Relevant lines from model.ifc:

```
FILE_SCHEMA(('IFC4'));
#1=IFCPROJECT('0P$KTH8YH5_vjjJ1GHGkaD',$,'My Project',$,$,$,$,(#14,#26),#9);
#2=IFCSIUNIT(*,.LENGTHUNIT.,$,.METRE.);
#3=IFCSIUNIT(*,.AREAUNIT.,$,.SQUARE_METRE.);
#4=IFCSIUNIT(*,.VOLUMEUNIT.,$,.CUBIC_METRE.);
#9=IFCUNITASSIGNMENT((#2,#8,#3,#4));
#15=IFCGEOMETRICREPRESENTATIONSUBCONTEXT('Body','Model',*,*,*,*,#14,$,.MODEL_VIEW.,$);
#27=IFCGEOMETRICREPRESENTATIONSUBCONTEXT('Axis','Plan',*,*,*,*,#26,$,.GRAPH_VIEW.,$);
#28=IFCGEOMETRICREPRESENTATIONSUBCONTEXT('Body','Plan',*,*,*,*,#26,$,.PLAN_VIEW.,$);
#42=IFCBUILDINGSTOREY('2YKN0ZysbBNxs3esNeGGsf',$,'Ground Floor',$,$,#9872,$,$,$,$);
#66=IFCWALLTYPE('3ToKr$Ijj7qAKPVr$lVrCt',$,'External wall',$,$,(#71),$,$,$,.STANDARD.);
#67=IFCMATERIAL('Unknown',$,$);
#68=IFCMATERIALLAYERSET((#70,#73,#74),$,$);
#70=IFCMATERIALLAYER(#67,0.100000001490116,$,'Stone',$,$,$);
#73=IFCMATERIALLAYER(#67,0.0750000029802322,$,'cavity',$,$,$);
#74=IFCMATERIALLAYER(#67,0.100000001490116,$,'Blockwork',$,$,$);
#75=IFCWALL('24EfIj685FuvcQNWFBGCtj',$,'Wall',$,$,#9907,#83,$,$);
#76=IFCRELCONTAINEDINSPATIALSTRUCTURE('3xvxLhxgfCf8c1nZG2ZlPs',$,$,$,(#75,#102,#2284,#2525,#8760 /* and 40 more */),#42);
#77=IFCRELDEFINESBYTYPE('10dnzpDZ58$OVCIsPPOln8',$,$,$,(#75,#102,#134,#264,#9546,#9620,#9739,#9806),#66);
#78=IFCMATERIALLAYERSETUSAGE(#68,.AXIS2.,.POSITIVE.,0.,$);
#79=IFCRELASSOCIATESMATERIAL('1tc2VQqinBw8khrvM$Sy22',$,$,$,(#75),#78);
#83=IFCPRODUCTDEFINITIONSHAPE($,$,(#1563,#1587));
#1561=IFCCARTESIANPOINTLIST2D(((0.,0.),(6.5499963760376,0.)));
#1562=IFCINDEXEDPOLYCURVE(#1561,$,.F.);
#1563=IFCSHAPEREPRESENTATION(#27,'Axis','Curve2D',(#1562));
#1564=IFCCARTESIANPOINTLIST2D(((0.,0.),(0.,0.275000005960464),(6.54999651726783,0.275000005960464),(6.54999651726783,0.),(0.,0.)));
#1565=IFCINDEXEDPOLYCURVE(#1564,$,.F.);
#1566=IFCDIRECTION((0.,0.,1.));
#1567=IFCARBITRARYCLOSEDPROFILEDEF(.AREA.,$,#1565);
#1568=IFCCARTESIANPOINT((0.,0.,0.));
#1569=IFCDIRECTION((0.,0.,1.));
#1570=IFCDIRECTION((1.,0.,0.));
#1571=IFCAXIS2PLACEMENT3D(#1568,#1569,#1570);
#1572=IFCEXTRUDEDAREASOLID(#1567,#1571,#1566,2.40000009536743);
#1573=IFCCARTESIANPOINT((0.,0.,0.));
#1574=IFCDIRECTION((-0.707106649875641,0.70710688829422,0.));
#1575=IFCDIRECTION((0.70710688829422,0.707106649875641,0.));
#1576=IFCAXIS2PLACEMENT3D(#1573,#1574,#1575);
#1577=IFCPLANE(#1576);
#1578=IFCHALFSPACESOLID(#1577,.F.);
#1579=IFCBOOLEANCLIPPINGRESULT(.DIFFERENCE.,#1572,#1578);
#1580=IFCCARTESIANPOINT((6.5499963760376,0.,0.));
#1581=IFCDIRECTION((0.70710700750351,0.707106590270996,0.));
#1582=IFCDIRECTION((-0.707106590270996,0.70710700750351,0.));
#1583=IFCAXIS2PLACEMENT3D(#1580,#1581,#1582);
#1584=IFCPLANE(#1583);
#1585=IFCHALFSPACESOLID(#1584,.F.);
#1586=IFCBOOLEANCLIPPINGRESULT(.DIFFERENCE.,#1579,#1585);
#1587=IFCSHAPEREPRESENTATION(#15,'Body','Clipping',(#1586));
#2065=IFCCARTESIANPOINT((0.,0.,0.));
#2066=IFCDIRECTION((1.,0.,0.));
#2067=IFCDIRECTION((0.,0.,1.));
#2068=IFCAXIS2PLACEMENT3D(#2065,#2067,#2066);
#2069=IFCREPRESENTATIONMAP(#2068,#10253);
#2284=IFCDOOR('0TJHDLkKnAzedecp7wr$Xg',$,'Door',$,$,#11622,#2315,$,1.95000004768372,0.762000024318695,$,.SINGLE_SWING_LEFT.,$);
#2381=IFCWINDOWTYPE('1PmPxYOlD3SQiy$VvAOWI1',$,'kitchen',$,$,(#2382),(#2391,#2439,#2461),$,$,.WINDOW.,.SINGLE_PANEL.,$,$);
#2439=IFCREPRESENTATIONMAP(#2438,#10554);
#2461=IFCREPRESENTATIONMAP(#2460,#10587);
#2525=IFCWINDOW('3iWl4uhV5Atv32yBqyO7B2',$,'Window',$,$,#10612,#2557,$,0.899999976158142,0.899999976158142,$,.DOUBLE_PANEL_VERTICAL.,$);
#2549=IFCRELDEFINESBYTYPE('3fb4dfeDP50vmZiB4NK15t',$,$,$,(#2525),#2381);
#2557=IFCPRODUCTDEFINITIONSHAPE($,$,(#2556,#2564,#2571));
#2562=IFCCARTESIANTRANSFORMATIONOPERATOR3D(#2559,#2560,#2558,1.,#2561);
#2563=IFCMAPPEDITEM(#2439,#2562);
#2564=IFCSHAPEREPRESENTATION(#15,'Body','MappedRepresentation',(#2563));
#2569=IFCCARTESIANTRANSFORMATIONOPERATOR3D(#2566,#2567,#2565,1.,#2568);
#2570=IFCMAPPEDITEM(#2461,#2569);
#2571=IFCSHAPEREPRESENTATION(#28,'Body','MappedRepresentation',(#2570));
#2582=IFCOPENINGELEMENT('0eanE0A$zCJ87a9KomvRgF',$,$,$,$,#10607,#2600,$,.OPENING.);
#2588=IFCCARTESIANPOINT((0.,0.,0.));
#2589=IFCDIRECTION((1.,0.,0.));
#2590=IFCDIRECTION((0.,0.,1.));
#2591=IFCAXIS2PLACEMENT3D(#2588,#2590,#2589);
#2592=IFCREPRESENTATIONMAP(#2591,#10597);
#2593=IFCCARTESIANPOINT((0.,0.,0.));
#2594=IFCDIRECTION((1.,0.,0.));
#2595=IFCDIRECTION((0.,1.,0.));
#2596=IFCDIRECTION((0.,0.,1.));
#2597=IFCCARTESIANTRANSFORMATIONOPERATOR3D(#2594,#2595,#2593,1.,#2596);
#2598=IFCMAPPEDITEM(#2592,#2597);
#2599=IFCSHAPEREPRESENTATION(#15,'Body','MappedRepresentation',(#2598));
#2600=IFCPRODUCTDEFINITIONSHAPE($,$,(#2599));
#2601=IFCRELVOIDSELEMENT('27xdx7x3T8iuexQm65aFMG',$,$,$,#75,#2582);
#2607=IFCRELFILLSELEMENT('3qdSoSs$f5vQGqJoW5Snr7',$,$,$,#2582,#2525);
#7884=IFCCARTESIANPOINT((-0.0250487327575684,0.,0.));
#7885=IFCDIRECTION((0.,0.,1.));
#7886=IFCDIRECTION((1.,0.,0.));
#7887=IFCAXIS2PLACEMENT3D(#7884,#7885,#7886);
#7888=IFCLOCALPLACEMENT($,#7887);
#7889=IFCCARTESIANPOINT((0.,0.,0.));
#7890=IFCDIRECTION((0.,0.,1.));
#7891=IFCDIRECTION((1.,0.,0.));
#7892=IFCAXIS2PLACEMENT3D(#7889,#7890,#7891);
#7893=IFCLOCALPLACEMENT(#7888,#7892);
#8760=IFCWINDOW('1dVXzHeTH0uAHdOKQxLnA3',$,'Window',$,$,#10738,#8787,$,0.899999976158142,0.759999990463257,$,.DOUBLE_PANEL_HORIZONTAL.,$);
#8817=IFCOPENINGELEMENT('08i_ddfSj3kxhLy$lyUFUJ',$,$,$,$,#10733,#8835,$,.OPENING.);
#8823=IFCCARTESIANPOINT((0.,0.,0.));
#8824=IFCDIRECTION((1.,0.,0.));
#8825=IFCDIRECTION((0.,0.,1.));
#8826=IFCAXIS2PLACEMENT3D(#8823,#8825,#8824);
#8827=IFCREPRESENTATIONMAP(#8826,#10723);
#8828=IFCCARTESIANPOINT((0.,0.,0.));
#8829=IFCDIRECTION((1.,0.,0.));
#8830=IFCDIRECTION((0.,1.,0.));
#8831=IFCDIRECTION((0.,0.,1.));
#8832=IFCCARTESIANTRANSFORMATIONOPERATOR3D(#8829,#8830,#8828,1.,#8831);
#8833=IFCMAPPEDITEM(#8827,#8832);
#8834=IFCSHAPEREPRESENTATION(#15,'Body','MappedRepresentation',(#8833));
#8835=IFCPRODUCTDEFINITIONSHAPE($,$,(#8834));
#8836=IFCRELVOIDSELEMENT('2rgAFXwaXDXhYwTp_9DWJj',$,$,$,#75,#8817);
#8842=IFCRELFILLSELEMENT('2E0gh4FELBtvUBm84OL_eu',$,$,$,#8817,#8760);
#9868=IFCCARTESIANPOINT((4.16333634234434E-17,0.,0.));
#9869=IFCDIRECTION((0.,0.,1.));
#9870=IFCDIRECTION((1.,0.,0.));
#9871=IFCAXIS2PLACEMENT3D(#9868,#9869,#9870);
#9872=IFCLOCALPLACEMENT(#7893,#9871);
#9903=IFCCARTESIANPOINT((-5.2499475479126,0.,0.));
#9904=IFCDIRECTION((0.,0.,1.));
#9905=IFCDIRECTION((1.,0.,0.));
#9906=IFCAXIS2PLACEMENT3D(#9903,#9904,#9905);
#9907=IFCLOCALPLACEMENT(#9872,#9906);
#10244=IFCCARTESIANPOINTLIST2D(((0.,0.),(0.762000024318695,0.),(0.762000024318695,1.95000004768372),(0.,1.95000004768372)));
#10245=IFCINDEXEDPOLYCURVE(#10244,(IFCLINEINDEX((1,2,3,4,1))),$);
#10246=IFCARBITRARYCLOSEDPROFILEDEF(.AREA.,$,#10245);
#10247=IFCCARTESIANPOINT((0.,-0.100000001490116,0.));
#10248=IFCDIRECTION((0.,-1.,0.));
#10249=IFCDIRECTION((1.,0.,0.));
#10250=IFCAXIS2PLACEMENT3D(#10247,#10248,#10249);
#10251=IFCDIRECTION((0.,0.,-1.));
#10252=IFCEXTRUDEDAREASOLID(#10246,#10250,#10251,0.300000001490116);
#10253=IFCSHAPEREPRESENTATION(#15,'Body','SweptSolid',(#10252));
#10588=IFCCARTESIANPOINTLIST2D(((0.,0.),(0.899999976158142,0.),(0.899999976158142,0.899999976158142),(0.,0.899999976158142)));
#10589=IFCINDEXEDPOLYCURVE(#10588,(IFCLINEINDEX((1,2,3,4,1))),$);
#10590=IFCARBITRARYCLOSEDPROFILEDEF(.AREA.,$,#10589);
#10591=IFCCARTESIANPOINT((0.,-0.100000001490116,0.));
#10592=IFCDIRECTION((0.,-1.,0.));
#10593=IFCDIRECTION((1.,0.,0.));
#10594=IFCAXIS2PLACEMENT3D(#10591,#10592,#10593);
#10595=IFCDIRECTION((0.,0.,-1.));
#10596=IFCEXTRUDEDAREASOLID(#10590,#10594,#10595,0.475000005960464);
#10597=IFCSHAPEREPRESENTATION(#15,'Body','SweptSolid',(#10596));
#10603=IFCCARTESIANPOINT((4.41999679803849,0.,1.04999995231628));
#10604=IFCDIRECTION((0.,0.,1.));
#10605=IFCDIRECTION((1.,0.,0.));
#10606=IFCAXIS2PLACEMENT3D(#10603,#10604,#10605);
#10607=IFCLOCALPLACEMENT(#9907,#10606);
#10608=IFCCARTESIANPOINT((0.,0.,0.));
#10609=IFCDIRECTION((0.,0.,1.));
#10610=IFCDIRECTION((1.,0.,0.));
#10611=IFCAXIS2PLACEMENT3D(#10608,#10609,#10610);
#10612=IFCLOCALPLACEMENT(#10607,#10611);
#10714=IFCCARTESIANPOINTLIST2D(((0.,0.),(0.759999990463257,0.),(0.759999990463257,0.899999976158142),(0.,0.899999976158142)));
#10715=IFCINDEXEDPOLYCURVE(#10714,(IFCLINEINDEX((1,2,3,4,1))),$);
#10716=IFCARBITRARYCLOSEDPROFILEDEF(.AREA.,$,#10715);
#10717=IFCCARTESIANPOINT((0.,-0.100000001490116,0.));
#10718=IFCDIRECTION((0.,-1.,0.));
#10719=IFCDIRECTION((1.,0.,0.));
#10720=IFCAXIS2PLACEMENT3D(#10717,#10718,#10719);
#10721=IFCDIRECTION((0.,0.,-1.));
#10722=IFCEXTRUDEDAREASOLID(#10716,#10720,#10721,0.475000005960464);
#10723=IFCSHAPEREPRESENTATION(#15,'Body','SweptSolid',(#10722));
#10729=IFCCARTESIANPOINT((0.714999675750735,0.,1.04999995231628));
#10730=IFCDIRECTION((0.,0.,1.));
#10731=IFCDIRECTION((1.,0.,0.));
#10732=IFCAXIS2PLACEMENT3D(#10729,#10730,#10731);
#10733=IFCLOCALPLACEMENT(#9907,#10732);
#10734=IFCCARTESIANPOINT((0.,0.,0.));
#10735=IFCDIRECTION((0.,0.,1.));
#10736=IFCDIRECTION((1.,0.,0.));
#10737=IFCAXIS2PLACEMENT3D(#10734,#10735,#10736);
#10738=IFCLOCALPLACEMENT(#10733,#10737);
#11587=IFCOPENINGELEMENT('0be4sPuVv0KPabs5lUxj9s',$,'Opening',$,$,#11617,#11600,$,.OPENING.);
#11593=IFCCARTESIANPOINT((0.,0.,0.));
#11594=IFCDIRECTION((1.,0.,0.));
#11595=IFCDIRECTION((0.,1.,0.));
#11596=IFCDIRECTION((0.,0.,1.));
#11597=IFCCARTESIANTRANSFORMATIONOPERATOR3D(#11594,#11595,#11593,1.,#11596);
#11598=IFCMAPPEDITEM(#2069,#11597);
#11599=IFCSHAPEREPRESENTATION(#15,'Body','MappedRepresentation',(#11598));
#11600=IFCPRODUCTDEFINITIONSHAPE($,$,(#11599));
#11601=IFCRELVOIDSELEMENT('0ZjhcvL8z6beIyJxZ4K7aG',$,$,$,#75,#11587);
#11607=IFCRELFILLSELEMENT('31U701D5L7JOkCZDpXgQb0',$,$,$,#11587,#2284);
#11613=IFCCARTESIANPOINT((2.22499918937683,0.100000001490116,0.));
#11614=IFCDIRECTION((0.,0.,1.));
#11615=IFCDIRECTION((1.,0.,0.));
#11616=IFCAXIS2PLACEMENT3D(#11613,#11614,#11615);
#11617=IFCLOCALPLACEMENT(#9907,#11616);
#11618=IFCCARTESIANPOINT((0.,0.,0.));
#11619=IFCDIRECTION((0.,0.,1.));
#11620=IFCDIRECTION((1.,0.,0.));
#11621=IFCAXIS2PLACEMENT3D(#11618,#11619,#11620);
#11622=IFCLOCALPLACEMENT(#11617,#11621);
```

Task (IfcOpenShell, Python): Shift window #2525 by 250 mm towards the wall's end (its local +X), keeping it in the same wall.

```python
import ifcopenshell
import ifcopenshell.api.geometry
import ifcopenshell.util.placement
import ifcopenshell.util.unit

model = ifcopenshell.open("model.ifc")
unit_scale = ifcopenshell.util.unit.calculate_unit_scale(model)

window = model.by_id(2525)
opening = window.FillsVoids[0].RelatingOpeningElement
wall = opening.VoidsElements[0].RelatingBuildingElement

wall_matrix = ifcopenshell.util.placement.get_local_placement(wall.ObjectPlacement)
shift = wall_matrix[:3, 0] * 0.25 / unit_scale
before = ifcopenshell.util.placement.get_local_placement(window.ObjectPlacement)[:3, 3].copy()

# The window is placed relative to its opening, so it follows when the opening moves.
matrix = ifcopenshell.util.placement.get_local_placement(opening.ObjectPlacement)
matrix[:3, 3] += shift
ifcopenshell.api.geometry.edit_object_placement(
    model, product=opening, matrix=matrix, is_si=False, should_transform_children=True
)

after = ifcopenshell.util.placement.get_local_placement(window.ObjectPlacement)[:3, 3]
print("window moved by", (after - before).round(3) + 0.0)

model.write("model_edited.ifc")
```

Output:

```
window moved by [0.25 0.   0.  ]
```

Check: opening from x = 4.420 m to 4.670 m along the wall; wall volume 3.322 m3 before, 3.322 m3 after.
